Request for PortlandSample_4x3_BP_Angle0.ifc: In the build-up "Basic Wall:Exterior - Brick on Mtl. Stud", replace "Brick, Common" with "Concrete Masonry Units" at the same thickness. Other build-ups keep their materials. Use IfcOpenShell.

First a look at what the model holds.

```python
import ifcopenshell
import ifcopenshell.util.element

model = ifcopenshell.open("PortlandSample_4x3_BP_Angle0.ifc")
print(model.schema)
for layer_set in model.by_type("IfcMaterialLayerSet"):
    if layer_set.LayerSetName == "Basic Wall:Exterior - Brick on Mtl. Stud":
        for layer in layer_set.MaterialLayers:
            print(layer.id(), layer.Material and layer.Material.Name, layer.LayerThickness, sep=" | ")
        print(len(ifcopenshell.util.element.get_elements_by_material(model, layer_set)), "elements and types use it")
print(sorted(m.Name for m in model.by_type("IfcMaterial") if m.Name)[:60])
```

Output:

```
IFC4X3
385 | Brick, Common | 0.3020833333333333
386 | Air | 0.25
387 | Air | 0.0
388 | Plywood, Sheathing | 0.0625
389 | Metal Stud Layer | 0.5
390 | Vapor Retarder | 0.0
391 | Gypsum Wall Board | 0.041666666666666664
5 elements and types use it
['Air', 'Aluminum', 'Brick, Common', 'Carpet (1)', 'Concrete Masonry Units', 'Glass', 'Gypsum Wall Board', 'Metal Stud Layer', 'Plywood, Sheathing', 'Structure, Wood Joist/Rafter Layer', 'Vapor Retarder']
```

```python
import ifcopenshell
import ifcopenshell.api.material

model = ifcopenshell.open("PortlandSample_4x3_BP_Angle0.ifc")

layer_set = next(s for s in model.by_type("IfcMaterialLayerSet") if s.LayerSetName == "Basic Wall:Exterior - Brick on Mtl. Stud")
layer = next(l for l in layer_set.MaterialLayers if l.Material and l.Material.Name == "Brick, Common")
material = next(m for m in model.by_type("IfcMaterial") if m.Name == "Concrete Masonry Units")

# Point this one layer at the other material; renaming the old one would change it everywhere.
ifcopenshell.api.material.edit_layer(model, layer=layer, attributes={"Name": material.Name}, material=material)

print([l.Material.Name if l.Material else None for l in layer_set.MaterialLayers])

model.write("PortlandSample_4x3_BP_Angle0_edited.ifc")
```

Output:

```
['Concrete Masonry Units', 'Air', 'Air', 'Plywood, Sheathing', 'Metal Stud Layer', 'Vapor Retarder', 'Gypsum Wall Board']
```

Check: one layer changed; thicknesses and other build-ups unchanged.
